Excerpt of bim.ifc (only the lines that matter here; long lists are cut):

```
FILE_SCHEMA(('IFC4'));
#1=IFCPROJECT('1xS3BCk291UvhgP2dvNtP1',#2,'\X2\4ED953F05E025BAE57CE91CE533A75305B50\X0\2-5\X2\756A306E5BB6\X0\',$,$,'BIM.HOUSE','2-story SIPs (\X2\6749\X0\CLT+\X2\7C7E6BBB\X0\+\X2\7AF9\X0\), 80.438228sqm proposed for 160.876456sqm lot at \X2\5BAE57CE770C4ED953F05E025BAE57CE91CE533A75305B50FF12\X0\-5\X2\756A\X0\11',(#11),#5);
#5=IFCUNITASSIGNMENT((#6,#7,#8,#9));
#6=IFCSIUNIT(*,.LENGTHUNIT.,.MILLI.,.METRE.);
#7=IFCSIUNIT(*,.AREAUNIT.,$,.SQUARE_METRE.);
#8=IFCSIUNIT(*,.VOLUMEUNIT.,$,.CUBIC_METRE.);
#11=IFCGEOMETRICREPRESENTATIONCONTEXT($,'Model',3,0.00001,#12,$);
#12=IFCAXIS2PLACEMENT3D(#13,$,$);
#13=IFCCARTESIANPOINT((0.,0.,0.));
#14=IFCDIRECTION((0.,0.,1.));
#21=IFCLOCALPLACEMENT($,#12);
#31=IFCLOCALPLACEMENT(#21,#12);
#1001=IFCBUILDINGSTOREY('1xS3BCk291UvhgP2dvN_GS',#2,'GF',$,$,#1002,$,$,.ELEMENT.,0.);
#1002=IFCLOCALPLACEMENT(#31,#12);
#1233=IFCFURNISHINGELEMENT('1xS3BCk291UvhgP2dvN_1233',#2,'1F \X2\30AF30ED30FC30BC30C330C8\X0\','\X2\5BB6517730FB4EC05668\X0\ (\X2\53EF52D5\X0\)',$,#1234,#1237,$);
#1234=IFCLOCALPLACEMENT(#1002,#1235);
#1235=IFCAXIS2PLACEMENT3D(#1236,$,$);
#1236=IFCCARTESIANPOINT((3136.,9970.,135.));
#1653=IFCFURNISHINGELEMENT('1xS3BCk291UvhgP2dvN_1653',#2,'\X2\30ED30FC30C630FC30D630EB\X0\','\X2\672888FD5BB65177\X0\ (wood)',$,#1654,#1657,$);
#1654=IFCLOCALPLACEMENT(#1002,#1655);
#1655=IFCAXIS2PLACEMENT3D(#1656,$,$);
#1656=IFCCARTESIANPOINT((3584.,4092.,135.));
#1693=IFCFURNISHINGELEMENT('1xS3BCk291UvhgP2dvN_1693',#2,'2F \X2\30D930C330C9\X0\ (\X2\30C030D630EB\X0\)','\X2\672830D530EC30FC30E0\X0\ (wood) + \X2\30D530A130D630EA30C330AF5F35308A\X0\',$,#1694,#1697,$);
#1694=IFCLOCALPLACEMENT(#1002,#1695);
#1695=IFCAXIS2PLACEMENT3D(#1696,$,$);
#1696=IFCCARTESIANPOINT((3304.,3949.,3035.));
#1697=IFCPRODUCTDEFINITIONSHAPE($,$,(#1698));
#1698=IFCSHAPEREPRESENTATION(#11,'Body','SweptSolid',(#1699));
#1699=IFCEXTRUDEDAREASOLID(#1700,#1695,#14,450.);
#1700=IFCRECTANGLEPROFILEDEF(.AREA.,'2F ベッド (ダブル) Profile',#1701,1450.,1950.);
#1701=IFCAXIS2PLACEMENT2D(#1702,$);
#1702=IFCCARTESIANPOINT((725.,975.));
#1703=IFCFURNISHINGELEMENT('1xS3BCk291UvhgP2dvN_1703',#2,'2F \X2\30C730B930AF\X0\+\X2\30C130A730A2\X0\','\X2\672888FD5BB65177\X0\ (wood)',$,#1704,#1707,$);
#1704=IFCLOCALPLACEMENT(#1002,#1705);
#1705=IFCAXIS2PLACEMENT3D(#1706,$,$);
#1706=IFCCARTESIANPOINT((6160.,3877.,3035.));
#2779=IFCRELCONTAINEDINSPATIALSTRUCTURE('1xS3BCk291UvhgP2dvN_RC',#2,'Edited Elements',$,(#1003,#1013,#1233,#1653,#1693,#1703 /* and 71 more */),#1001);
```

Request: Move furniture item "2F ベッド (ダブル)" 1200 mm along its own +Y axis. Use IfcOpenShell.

```python
import ifcopenshell
import ifcopenshell.api.geometry
import ifcopenshell.util.placement

model = ifcopenshell.open("bim.ifc")

item = model.by_guid("1xS3BCk291UvhgP2dvN_1693")
matrix = ifcopenshell.util.placement.get_local_placement(item.ObjectPlacement)
matrix[:3, 3] += matrix[:3, 1] * 1200.0
ifcopenshell.api.geometry.edit_object_placement(model, product=item, matrix=matrix, is_si=False)

print(ifcopenshell.util.placement.get_local_placement(item.ObjectPlacement).round(3) + 0.0)

model.write("bim_edited.ifc")
```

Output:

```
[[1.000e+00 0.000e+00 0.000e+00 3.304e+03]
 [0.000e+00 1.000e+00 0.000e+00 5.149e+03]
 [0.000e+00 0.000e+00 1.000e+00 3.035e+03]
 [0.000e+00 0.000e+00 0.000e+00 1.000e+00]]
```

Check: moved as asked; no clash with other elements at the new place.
